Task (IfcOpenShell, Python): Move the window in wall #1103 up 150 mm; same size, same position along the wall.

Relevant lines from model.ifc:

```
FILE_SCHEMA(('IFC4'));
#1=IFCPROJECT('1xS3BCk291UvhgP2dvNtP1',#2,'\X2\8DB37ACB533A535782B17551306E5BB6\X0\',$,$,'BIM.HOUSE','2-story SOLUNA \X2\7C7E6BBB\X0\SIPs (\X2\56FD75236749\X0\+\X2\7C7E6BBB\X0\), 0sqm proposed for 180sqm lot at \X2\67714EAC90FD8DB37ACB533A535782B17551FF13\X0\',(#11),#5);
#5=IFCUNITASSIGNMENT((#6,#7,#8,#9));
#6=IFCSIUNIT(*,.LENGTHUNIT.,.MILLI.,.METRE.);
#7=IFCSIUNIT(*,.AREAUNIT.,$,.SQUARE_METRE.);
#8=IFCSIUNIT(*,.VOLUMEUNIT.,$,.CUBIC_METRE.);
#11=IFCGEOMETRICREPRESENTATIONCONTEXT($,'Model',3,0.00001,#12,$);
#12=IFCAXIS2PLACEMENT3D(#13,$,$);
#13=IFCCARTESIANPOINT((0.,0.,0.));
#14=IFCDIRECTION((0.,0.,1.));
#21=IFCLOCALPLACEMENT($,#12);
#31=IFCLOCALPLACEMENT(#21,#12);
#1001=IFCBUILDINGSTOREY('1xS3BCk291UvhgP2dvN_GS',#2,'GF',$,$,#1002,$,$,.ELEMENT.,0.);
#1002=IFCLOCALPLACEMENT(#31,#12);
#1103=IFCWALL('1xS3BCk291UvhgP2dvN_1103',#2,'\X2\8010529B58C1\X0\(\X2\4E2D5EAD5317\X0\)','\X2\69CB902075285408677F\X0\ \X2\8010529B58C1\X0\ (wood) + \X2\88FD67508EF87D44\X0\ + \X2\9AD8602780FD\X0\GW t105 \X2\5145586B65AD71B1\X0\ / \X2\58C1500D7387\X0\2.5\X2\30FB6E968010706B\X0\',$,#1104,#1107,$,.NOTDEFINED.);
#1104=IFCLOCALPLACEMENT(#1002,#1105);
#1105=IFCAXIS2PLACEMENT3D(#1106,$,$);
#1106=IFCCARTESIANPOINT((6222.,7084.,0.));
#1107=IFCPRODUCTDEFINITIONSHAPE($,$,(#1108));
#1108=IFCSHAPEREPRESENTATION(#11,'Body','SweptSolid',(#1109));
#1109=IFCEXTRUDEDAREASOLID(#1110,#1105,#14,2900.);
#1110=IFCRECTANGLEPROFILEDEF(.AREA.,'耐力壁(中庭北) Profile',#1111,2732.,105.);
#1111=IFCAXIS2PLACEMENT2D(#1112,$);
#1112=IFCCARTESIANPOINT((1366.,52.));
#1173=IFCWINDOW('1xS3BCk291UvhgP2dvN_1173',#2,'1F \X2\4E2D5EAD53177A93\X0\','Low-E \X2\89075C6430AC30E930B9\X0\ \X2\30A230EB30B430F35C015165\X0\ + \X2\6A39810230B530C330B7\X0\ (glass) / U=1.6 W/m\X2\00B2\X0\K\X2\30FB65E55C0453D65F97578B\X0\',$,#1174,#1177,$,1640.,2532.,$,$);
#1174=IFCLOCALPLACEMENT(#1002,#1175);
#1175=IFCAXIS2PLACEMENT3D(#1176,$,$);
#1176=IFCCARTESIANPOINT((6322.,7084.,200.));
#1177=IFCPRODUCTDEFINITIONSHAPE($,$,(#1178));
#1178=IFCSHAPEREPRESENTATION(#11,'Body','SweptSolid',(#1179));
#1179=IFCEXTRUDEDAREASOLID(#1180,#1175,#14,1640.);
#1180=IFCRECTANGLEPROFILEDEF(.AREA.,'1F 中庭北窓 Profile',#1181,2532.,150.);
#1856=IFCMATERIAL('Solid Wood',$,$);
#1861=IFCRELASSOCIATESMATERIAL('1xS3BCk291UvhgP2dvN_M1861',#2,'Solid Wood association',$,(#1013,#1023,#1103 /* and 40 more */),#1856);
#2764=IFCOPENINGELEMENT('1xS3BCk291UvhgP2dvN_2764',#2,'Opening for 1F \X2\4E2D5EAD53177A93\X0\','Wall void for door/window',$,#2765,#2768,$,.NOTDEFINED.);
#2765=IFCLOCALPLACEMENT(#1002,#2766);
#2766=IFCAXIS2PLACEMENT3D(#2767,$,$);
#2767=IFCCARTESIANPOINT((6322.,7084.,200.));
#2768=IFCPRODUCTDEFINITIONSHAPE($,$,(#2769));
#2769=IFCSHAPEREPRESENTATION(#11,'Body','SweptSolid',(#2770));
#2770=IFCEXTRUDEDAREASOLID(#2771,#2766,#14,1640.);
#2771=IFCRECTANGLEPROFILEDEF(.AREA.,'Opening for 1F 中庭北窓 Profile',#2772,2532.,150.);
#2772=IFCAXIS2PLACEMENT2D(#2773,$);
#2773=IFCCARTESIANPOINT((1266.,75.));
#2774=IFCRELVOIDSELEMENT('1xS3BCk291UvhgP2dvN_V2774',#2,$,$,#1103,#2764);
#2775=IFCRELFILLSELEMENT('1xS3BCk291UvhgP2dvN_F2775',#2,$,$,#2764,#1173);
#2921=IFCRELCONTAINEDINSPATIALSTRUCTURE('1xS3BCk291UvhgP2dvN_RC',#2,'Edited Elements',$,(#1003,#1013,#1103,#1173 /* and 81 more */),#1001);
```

```python
import numpy as np
import ifcopenshell
import ifcopenshell.api.geometry
import ifcopenshell.util.placement
import ifcopenshell.util.unit

model = ifcopenshell.open("model.ifc")
unit_scale = ifcopenshell.util.unit.calculate_unit_scale(model)

window = model.by_guid("1xS3BCk291UvhgP2dvN_1173")
opening = window.FillsVoids[0].RelatingOpeningElement
dz = 150.0

shift = np.array([0.0, 0.0, dz])
# The window is not placed relative to its opening, so move both.
for product in (opening, window):
    matrix = ifcopenshell.util.placement.get_local_placement(product.ObjectPlacement)
    matrix[:3, 3] += shift
    ifcopenshell.api.geometry.edit_object_placement(model, product=product, matrix=matrix, is_si=False)

print(f"moved by {dz * unit_scale:+.3f} m")

model.write("model_updated.ifc")
```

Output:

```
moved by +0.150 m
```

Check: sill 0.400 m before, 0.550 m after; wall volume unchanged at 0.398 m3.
